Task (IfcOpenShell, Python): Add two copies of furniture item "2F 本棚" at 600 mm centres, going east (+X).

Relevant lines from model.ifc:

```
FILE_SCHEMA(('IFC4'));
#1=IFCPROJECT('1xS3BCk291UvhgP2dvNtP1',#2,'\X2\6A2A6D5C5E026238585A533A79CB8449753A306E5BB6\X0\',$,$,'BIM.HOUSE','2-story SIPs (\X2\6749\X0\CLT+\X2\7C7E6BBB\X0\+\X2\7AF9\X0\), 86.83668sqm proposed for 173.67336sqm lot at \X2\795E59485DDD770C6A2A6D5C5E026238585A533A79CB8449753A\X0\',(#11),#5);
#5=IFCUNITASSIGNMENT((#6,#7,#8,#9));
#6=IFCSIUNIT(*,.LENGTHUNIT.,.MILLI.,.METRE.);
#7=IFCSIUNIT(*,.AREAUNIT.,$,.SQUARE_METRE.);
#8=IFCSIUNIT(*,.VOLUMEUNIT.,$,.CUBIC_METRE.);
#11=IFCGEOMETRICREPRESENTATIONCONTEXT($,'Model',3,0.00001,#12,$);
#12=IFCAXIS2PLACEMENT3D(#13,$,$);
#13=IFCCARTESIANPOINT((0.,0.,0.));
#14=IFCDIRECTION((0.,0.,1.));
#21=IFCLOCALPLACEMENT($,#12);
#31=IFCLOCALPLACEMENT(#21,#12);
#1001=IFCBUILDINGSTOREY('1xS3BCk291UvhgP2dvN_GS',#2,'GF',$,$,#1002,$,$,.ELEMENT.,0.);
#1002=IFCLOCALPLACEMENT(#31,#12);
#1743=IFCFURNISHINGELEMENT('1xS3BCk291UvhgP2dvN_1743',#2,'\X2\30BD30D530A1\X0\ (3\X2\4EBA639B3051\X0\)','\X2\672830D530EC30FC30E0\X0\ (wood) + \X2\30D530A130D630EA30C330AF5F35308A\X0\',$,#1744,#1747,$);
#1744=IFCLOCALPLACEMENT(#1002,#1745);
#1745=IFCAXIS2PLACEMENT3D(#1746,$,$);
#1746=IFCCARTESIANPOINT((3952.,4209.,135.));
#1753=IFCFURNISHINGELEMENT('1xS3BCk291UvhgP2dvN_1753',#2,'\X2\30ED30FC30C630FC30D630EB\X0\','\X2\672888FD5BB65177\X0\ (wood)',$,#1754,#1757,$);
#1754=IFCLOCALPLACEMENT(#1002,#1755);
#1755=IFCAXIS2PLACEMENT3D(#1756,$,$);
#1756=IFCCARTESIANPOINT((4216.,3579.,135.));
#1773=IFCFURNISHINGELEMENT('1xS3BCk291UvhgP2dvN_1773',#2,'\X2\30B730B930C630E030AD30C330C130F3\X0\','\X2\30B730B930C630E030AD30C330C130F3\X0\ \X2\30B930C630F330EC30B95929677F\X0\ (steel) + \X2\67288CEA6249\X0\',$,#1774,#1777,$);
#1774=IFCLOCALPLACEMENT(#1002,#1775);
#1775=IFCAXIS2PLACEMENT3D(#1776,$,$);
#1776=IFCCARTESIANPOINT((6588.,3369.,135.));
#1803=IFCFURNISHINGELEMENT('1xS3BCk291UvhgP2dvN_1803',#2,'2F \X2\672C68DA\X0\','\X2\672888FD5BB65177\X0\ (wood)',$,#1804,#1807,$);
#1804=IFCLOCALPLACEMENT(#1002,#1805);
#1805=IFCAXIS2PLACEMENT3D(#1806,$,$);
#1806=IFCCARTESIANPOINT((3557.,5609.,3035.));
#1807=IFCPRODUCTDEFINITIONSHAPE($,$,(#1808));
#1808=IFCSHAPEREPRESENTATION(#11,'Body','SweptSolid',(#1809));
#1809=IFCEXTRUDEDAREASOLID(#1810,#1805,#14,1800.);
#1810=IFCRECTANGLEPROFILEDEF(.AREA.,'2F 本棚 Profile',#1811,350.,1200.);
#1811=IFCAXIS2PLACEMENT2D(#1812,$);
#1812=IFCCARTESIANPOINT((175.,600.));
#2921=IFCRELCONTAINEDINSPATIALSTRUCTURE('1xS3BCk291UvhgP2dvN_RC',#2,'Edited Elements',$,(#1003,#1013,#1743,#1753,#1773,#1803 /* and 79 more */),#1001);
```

```python
import numpy as np
import ifcopenshell
import ifcopenshell.api.geometry
import ifcopenshell.api.root
import ifcopenshell.util.element
import ifcopenshell.util.placement
import ifcopenshell.util.unit

model = ifcopenshell.open("model.ifc")
unit_scale = ifcopenshell.util.unit.calculate_unit_scale(model)


def reuse_history(source, copy):
    """copy_class also copies each property set's owner history, people and application; keep the originals."""
    for rel in copy.IsDefinedBy:
        if rel.is_a("IfcRelDefinesByProperties") and (history := rel.RelatingPropertyDefinition.OwnerHistory):
            rel.RelatingPropertyDefinition.OwnerHistory = source.OwnerHistory
            ifcopenshell.util.element.remove_deep2(model, history)


source = model.by_guid("1xS3BCk291UvhgP2dvN_1803")
base = ifcopenshell.util.placement.get_local_placement(source.ObjectPlacement)
step = np.array([1.0, 0.0, 0.0]) * 0.6 / unit_scale

for i in range(1, 3):
    copy = ifcopenshell.api.root.copy_class(model, product=source)
    copy.Representation = ifcopenshell.util.element.copy_deep(
        model, source.Representation, exclude=["IfcGeometricRepresentationContext", "IfcRepresentationMap"]
    )
    reuse_history(source, copy)
    matrix = base.copy()
    matrix[:3, 3] += i * step
    print("added at", matrix[:3, 3].round(3) + 0.0)
    ifcopenshell.api.geometry.edit_object_placement(model, product=copy, matrix=matrix, is_si=False)

model.write("model_rev.ifc")
```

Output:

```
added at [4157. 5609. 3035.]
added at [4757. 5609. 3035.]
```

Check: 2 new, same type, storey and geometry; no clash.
